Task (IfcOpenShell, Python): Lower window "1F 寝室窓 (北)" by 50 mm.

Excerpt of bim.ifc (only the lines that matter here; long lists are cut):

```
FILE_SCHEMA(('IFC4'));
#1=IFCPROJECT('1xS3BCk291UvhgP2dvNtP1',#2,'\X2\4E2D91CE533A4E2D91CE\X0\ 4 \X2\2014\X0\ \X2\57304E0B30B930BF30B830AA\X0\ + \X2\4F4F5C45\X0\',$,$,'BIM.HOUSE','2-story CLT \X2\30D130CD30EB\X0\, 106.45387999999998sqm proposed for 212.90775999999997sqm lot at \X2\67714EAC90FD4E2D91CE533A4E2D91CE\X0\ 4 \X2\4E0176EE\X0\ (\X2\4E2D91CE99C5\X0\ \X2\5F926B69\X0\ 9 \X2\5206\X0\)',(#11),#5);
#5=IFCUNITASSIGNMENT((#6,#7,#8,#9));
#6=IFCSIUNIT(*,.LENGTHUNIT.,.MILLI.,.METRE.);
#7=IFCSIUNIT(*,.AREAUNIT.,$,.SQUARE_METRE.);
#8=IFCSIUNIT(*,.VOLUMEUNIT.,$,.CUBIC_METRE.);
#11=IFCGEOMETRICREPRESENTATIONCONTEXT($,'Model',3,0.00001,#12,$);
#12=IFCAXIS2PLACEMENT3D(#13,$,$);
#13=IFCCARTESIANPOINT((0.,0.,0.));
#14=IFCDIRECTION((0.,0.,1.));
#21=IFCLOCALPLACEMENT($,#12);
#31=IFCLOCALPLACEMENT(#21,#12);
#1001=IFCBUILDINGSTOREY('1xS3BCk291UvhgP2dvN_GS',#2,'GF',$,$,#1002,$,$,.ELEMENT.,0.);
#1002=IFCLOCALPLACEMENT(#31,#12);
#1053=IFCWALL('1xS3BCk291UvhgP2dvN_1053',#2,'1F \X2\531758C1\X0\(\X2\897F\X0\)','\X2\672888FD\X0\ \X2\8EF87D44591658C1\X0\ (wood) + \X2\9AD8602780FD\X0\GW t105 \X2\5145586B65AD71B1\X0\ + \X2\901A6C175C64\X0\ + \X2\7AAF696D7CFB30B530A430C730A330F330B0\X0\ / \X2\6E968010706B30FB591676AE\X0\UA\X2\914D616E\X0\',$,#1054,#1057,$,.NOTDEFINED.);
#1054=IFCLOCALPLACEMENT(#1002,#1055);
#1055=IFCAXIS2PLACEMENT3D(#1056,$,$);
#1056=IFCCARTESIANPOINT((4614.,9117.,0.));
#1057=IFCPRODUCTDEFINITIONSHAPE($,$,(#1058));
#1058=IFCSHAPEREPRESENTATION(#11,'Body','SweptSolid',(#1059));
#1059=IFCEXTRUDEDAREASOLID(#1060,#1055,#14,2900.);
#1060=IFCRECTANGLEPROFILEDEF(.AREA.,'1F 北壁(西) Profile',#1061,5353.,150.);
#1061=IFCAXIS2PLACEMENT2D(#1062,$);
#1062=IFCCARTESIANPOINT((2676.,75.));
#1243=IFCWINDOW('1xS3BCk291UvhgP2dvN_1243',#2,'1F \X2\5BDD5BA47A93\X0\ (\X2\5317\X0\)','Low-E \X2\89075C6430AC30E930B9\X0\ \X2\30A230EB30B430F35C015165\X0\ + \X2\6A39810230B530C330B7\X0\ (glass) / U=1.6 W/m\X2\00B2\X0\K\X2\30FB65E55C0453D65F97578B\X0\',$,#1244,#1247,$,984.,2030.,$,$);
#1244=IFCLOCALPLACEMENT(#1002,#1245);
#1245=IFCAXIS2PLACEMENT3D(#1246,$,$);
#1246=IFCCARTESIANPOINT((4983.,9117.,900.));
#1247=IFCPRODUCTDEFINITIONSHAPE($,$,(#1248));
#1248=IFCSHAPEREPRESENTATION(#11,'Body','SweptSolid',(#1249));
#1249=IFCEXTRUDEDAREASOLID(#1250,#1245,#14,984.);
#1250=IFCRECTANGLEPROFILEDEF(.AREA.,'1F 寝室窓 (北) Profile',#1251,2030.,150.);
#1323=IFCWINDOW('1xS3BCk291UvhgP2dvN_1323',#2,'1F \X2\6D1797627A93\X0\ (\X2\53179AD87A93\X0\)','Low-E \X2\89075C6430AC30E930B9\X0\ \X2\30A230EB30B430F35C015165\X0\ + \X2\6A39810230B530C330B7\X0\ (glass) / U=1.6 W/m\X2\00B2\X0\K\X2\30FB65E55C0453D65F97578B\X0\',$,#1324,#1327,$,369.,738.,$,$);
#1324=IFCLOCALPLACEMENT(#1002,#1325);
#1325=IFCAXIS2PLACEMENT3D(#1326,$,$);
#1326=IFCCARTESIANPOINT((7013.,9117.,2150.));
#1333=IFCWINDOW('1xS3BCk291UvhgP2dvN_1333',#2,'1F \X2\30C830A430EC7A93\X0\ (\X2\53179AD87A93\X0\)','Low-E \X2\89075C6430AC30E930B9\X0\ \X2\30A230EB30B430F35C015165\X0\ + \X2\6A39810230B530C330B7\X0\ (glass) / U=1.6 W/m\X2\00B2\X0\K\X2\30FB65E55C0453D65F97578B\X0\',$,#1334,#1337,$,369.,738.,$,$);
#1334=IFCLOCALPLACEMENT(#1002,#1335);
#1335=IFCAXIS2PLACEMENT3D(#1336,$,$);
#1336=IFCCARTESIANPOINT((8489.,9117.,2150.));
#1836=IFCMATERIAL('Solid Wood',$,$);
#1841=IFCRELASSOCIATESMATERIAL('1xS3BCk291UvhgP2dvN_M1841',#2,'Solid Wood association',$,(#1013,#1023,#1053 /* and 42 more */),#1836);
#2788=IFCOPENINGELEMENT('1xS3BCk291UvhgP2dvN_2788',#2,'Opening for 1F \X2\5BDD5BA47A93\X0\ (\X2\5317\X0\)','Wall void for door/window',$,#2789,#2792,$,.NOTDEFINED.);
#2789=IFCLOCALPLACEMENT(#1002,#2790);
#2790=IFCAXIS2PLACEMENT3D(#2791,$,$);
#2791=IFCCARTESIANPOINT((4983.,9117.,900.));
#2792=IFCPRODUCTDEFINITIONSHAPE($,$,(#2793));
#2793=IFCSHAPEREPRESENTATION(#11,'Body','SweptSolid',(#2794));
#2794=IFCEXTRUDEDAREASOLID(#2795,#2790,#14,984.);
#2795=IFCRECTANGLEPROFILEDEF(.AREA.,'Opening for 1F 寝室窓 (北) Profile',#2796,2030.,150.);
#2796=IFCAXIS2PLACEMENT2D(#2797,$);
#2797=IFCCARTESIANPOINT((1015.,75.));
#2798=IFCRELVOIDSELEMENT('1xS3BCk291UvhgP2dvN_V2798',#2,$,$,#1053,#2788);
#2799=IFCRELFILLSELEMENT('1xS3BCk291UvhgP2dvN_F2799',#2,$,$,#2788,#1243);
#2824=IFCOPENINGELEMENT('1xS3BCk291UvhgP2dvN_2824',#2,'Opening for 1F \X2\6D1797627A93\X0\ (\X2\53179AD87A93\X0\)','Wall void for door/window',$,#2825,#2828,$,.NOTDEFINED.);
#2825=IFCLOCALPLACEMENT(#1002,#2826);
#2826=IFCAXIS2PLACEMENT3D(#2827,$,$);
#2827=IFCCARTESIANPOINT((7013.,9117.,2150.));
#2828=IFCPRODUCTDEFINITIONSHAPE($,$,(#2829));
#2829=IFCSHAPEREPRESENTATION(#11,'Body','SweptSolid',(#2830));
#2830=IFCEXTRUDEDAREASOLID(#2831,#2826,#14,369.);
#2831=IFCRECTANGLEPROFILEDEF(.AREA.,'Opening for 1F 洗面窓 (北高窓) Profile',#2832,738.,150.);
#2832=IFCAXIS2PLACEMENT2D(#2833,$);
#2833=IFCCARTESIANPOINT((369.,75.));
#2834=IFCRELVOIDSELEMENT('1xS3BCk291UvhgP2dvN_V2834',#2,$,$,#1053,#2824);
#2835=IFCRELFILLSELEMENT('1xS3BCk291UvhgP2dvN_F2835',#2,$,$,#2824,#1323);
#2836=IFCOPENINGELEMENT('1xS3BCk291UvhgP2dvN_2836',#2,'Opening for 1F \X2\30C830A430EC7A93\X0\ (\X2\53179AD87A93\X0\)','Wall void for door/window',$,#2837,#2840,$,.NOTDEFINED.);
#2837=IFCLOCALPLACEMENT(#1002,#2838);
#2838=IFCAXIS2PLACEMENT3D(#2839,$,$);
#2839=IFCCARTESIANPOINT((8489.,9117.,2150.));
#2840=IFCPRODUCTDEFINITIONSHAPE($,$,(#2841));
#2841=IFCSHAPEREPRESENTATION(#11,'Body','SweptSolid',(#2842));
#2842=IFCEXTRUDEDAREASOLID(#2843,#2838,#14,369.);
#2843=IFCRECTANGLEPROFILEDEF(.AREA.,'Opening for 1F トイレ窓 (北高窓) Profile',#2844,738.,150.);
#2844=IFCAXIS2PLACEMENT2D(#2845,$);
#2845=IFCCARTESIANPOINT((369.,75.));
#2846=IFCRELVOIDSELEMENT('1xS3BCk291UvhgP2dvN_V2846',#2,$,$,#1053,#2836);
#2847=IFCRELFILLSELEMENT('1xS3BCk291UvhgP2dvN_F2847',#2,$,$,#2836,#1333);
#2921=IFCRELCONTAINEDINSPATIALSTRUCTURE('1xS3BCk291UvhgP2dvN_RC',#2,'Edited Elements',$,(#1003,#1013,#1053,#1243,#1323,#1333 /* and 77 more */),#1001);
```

```python
import numpy as np
import ifcopenshell
import ifcopenshell.api.geometry
import ifcopenshell.util.placement
import ifcopenshell.util.unit

model = ifcopenshell.open("bim.ifc")
unit_scale = ifcopenshell.util.unit.calculate_unit_scale(model)

window = model.by_guid("1xS3BCk291UvhgP2dvN_1243")
opening = window.FillsVoids[0].RelatingOpeningElement
dz = -0.05 / unit_scale

shift = np.array([0.0, 0.0, dz])
# The window is not placed relative to its opening, so move both.
for product in (opening, window):
    matrix = ifcopenshell.util.placement.get_local_placement(product.ObjectPlacement)
    matrix[:3, 3] += shift
    ifcopenshell.api.geometry.edit_object_placement(model, product=product, matrix=matrix, is_si=False)

print(f"moved by {dz * unit_scale:+.3f} m")

model.write("bim-out.ifc")
```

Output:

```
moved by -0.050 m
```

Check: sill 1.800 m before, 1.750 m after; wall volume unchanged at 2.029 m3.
